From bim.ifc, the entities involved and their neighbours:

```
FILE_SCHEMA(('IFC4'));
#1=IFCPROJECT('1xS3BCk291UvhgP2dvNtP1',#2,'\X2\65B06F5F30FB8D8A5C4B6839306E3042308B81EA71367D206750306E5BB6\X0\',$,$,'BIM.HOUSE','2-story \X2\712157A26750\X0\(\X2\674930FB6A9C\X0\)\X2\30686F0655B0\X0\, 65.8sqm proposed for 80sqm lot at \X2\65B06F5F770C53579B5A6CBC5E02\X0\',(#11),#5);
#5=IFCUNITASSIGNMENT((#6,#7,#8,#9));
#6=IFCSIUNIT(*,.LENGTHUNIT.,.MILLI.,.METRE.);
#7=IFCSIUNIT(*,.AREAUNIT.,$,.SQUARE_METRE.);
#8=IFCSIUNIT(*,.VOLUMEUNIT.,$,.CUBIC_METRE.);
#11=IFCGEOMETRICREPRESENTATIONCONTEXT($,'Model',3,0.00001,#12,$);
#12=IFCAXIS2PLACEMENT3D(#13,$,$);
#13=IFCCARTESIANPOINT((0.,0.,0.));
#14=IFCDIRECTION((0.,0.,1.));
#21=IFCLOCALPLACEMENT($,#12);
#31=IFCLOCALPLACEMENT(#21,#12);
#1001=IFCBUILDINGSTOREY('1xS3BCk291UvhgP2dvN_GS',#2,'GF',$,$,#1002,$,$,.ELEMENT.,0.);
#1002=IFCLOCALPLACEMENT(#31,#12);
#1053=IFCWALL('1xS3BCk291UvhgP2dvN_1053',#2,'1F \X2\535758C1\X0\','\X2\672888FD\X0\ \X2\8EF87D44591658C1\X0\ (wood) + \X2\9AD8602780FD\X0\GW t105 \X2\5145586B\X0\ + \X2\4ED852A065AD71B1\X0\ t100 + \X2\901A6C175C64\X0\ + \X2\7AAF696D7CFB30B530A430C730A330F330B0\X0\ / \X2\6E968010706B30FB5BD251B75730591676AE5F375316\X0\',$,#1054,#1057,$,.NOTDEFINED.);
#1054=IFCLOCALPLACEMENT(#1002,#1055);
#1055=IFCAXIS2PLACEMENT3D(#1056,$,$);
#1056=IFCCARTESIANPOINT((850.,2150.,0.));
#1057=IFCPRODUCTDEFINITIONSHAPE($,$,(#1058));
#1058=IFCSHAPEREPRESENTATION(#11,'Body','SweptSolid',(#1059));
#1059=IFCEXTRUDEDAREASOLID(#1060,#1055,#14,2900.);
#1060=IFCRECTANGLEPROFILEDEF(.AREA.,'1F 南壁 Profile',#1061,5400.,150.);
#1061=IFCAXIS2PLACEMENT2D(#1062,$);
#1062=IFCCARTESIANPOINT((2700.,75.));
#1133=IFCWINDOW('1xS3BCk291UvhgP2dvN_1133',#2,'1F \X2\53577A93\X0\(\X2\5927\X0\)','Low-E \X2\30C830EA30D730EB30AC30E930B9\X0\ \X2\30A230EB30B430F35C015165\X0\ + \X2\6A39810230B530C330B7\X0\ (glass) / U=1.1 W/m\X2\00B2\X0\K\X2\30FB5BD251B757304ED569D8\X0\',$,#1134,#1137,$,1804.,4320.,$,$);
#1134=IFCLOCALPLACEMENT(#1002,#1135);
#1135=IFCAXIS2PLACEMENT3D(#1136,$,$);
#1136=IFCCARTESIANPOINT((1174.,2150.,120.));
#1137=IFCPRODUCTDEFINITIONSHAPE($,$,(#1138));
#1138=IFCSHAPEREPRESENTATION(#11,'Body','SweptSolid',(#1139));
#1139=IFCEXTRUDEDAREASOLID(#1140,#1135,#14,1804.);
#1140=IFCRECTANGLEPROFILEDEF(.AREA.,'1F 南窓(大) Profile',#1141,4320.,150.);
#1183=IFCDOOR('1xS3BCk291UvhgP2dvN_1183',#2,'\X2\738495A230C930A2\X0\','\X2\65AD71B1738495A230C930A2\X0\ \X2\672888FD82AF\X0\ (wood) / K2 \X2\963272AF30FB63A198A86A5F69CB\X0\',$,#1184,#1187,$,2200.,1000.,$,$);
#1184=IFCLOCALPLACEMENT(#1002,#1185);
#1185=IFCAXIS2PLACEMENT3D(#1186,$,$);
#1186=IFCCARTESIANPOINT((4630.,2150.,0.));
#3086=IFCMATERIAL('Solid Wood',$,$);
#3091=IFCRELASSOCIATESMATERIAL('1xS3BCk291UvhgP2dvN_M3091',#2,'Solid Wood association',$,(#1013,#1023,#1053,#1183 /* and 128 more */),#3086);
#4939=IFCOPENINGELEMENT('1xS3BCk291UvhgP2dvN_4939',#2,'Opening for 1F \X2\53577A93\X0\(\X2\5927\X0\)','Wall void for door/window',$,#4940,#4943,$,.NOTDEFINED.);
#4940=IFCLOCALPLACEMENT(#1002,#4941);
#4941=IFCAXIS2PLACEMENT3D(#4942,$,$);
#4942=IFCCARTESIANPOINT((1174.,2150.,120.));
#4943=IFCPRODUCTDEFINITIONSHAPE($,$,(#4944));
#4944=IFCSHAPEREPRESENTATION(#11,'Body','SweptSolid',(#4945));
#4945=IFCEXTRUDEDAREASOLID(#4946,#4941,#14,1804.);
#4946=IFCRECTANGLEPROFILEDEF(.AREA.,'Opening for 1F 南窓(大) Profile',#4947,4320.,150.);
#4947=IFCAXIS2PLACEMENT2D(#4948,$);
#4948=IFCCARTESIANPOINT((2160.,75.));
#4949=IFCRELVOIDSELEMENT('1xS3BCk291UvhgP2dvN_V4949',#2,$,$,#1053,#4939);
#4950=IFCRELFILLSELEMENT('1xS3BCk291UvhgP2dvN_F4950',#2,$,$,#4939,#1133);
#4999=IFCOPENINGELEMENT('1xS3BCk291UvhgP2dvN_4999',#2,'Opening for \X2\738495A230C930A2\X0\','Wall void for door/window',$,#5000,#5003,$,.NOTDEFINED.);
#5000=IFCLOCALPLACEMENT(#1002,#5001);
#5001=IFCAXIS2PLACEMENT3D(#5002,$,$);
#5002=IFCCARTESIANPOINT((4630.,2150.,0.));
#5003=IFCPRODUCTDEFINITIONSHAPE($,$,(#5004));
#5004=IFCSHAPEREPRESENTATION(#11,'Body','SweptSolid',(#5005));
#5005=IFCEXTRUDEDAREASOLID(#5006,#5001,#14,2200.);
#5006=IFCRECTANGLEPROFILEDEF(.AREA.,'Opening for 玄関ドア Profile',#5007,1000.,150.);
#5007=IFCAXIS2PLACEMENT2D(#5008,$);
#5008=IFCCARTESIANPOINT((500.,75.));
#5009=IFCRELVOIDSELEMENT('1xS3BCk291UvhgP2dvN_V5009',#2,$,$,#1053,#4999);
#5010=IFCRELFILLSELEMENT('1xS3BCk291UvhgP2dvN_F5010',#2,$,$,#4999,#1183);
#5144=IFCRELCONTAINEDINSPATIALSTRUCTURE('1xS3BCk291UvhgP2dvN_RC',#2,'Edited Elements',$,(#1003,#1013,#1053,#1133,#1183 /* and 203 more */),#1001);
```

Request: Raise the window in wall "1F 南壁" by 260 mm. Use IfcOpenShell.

```python
import numpy as np
import ifcopenshell
import ifcopenshell.api.geometry
import ifcopenshell.util.placement
import ifcopenshell.util.unit

model = ifcopenshell.open("bim.ifc")
unit_scale = ifcopenshell.util.unit.calculate_unit_scale(model)

window = model.by_id(1133)
opening = window.FillsVoids[0].RelatingOpeningElement
dz = 0.26 / unit_scale

shift = np.array([0.0, 0.0, dz])
# The window is not placed relative to its opening, so move both.
for product in (opening, window):
    matrix = ifcopenshell.util.placement.get_local_placement(product.ObjectPlacement)
    matrix[:3, 3] += shift
    ifcopenshell.api.geometry.edit_object_placement(model, product=product, matrix=matrix, is_si=False)

print(f"moved by {dz * unit_scale:+.3f} m")

model.write("bim_rev.ifc")
```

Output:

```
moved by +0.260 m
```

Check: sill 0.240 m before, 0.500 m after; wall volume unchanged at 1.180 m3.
